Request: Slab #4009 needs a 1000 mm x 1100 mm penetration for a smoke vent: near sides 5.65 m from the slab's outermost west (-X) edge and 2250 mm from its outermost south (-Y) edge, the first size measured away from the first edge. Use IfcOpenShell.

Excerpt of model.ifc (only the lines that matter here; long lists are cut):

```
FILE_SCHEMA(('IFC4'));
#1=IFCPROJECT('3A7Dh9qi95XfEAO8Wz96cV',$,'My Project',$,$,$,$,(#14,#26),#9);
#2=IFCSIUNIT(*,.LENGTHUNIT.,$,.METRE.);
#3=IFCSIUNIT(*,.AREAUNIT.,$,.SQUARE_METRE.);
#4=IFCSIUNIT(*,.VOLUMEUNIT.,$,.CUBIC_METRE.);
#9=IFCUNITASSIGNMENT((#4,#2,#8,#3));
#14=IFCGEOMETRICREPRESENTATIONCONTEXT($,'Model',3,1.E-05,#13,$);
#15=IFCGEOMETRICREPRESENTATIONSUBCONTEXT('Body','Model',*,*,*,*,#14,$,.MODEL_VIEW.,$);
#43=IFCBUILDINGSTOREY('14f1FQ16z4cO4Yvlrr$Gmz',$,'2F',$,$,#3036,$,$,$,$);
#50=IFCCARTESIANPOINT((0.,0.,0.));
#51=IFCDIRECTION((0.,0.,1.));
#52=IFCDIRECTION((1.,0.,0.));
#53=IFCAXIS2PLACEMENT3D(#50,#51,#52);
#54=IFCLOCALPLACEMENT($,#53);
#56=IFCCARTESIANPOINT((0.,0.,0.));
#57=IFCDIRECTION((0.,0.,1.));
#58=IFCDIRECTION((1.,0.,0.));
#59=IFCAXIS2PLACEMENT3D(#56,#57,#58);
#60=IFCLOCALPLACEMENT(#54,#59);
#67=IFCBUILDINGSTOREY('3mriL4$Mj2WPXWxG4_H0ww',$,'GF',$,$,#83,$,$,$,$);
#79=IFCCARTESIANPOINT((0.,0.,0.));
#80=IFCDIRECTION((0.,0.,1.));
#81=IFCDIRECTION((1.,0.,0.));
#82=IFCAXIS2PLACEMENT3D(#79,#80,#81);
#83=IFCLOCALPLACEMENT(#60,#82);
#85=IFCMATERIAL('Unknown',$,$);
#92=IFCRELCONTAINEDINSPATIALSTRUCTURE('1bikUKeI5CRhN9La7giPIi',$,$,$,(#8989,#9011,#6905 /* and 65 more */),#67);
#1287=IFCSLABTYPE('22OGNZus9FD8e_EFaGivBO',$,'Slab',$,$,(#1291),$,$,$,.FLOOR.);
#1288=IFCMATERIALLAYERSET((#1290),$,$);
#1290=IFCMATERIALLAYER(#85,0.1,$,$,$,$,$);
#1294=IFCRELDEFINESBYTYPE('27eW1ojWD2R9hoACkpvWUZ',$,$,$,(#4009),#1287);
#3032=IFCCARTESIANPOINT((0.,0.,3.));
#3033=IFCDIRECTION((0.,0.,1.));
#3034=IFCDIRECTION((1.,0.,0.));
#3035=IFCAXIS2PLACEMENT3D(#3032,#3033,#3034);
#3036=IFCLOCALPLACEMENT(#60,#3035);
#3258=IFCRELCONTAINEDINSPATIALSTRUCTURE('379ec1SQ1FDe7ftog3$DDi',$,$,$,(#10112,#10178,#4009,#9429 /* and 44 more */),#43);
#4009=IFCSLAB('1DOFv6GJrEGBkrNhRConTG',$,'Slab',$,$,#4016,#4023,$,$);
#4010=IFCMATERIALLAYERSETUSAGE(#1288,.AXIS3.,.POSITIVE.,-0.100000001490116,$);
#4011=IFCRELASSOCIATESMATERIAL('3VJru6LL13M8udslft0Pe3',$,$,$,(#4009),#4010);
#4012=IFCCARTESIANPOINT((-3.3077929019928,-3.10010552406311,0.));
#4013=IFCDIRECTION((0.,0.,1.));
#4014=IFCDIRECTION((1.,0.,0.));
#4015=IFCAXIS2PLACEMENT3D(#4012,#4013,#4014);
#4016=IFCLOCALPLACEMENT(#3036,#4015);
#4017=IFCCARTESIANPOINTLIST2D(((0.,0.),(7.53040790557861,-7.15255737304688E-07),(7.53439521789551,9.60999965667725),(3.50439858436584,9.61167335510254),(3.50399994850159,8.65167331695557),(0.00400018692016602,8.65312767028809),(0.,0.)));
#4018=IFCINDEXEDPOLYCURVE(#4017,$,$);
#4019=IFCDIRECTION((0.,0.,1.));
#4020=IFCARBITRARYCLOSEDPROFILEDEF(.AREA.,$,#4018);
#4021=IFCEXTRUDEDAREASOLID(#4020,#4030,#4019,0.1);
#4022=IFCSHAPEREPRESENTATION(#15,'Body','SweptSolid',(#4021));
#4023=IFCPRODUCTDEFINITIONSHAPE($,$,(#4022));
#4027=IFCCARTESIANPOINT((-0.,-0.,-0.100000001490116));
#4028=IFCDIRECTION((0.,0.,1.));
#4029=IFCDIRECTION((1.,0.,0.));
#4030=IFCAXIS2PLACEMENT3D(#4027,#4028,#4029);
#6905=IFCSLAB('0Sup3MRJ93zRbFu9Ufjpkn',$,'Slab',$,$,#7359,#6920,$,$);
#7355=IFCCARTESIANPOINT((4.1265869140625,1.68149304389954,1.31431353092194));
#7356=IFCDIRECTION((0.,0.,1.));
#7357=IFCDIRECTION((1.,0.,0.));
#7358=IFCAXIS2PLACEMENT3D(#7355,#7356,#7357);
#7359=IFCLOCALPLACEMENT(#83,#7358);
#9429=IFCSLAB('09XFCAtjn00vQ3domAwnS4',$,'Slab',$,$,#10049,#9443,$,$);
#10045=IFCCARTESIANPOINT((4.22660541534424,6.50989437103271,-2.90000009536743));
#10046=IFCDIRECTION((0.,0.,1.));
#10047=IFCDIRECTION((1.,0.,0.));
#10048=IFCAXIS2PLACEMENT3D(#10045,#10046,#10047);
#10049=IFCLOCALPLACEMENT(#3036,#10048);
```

```python
import numpy as np
import ifcopenshell
import ifcopenshell.api.feature
import ifcopenshell.api.geometry
import ifcopenshell.api.root
import ifcopenshell.geom
import ifcopenshell.util.placement
import ifcopenshell.util.representation
import ifcopenshell.util.shape
import ifcopenshell.util.unit

model = ifcopenshell.open("model.ifc")
unit_scale = ifcopenshell.util.unit.calculate_unit_scale(model)
settings = ifcopenshell.geom.settings()


def volume(element):
    """Net volume in cubic metres, openings subtracted."""
    shape = ifcopenshell.geom.create_shape(settings, element)
    return ifcopenshell.util.shape.get_volume(shape.geometry)


slab = model.by_guid("1DOFv6GJrEGBkrNhRConTG")
before = volume(slab)

# Extent in the slab's own axes, in metres. The edges named are its -X and -Y sides.
slab_shape = ifcopenshell.geom.create_shape(settings, slab)
vertices = ifcopenshell.util.shape.get_vertices(slab_shape.geometry)
x_min, y_min, bottom = vertices.min(axis=0)
top = vertices[:, 2].max()

opening = ifcopenshell.api.root.create_entity(model, ifc_class="IfcOpeningElement", name="Smoke vent opening", predefined_type="OPENING")
context = ifcopenshell.util.representation.get_context(model, "Model", "Body", "MODEL_VIEW")
width, depth = 1, 1.1
outline = [(0.0, 0.0), (width, 0.0), (width, depth), (0.0, depth), (0.0, 0.0)]
# Overshoot both faces by 50 mm so the cut is clean.
shape = ifcopenshell.api.geometry.add_slab_representation(
    model, context=context, depth=top - bottom + 0.1, polyline=outline
)
ifcopenshell.api.geometry.assign_representation(model, product=opening, representation=shape)

matrix = ifcopenshell.util.placement.get_local_placement(slab.ObjectPlacement)
matrix[:, 3] = matrix @ np.append(np.array([x_min + 5.65, y_min + 2.25, bottom - 0.05]) / unit_scale, 1.0)
ifcopenshell.api.geometry.edit_object_placement(model, product=opening, matrix=matrix, is_si=False)
ifcopenshell.api.feature.add_feature(model, feature=opening, element=slab)

after = volume(slab)

print(f"slab volume {before:.3f} -> {after:.3f} m3")

model.write("model_rev.ifc")
```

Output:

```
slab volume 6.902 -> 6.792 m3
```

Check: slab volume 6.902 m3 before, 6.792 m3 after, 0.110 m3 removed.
